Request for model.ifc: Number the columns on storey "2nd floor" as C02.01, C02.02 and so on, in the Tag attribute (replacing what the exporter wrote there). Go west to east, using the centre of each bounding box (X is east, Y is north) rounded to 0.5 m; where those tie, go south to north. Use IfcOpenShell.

First a look at what the model holds.

```python
import ifcopenshell
import ifcopenshell.util.element
import ifcopenshell.util.placement

model = ifcopenshell.open("model.ifc")
print(model.schema)
storey = next(s for s in model.by_type("IfcBuildingStorey") if s.Name == "2nd floor")
columns = [e for e in ifcopenshell.util.element.get_decomposition(storey) if e.is_a("IfcColumn")]
for e in sorted(columns, key=lambda e: e.id()):
    origin = ifcopenshell.util.placement.get_local_placement(e.ObjectPlacement)[:3, 3]
    print(e.id(), e.Tag, e.Name, origin.round(2) + 0.0, sep=" | ")
```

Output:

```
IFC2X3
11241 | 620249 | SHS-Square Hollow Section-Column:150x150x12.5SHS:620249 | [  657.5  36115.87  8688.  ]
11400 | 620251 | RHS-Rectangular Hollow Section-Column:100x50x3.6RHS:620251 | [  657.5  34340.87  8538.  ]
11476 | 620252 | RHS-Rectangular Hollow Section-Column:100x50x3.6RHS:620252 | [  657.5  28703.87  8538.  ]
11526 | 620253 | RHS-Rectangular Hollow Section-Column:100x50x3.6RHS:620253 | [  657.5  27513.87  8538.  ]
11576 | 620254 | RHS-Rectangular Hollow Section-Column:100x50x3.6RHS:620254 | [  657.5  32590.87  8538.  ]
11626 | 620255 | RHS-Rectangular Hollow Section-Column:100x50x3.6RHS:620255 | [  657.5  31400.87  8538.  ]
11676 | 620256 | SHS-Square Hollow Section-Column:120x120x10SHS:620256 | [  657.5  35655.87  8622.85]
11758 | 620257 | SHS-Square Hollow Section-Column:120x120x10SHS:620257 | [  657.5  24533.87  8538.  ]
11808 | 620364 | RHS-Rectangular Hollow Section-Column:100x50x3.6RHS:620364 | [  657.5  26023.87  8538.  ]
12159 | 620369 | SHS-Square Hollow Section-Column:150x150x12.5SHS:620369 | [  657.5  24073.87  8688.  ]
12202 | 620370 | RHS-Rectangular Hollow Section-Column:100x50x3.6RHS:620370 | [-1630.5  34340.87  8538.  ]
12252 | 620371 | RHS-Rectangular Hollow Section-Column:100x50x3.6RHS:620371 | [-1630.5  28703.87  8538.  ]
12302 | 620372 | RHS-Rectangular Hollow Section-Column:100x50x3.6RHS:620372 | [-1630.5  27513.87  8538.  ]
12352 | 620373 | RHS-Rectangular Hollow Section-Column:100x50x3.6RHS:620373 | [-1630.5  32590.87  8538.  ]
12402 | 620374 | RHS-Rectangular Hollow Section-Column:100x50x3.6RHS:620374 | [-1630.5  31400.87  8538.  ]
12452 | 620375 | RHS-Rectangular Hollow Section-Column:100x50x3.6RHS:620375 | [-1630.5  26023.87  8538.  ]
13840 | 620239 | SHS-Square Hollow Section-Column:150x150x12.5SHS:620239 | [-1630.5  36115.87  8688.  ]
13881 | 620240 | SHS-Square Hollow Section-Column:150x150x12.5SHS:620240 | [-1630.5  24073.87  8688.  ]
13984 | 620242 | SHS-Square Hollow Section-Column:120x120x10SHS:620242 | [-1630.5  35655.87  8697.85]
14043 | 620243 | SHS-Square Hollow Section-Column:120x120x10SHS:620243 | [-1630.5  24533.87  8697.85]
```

```python
import ifcopenshell
import ifcopenshell.geom
import ifcopenshell.util.element
import ifcopenshell.util.shape

model = ifcopenshell.open("model.ifc")
settings = ifcopenshell.geom.settings()
settings.set("use-world-coords", True)


def centre(element):
    shape = ifcopenshell.geom.create_shape(settings, element)
    return ifcopenshell.util.shape.get_bbox_centroid(shape.geometry)


storey = next(s for s in model.by_type("IfcBuildingStorey") if s.Name == "2nd floor")
columns = [e for e in ifcopenshell.util.element.get_decomposition(storey) if e.is_a("IfcColumn")]

# Insertion points can sit at a corner or the storey origin, so sort by the geometry (in metres).
centres = {e: centre(e) for e in columns}
columns.sort(key=lambda e: (round(centres[e][0] / 0.5), centres[e][1]))

for i, e in enumerate(columns, start=1):
    number = f"C02.{i:02d}"
    e.Tag = number
    print(e.id(), number)

model.write("model_rev.ifc")
```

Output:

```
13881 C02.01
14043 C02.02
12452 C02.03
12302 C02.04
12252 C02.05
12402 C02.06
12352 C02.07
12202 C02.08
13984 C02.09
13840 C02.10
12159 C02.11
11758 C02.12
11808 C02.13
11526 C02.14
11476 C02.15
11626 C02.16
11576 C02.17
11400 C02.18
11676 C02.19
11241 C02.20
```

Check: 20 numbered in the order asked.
